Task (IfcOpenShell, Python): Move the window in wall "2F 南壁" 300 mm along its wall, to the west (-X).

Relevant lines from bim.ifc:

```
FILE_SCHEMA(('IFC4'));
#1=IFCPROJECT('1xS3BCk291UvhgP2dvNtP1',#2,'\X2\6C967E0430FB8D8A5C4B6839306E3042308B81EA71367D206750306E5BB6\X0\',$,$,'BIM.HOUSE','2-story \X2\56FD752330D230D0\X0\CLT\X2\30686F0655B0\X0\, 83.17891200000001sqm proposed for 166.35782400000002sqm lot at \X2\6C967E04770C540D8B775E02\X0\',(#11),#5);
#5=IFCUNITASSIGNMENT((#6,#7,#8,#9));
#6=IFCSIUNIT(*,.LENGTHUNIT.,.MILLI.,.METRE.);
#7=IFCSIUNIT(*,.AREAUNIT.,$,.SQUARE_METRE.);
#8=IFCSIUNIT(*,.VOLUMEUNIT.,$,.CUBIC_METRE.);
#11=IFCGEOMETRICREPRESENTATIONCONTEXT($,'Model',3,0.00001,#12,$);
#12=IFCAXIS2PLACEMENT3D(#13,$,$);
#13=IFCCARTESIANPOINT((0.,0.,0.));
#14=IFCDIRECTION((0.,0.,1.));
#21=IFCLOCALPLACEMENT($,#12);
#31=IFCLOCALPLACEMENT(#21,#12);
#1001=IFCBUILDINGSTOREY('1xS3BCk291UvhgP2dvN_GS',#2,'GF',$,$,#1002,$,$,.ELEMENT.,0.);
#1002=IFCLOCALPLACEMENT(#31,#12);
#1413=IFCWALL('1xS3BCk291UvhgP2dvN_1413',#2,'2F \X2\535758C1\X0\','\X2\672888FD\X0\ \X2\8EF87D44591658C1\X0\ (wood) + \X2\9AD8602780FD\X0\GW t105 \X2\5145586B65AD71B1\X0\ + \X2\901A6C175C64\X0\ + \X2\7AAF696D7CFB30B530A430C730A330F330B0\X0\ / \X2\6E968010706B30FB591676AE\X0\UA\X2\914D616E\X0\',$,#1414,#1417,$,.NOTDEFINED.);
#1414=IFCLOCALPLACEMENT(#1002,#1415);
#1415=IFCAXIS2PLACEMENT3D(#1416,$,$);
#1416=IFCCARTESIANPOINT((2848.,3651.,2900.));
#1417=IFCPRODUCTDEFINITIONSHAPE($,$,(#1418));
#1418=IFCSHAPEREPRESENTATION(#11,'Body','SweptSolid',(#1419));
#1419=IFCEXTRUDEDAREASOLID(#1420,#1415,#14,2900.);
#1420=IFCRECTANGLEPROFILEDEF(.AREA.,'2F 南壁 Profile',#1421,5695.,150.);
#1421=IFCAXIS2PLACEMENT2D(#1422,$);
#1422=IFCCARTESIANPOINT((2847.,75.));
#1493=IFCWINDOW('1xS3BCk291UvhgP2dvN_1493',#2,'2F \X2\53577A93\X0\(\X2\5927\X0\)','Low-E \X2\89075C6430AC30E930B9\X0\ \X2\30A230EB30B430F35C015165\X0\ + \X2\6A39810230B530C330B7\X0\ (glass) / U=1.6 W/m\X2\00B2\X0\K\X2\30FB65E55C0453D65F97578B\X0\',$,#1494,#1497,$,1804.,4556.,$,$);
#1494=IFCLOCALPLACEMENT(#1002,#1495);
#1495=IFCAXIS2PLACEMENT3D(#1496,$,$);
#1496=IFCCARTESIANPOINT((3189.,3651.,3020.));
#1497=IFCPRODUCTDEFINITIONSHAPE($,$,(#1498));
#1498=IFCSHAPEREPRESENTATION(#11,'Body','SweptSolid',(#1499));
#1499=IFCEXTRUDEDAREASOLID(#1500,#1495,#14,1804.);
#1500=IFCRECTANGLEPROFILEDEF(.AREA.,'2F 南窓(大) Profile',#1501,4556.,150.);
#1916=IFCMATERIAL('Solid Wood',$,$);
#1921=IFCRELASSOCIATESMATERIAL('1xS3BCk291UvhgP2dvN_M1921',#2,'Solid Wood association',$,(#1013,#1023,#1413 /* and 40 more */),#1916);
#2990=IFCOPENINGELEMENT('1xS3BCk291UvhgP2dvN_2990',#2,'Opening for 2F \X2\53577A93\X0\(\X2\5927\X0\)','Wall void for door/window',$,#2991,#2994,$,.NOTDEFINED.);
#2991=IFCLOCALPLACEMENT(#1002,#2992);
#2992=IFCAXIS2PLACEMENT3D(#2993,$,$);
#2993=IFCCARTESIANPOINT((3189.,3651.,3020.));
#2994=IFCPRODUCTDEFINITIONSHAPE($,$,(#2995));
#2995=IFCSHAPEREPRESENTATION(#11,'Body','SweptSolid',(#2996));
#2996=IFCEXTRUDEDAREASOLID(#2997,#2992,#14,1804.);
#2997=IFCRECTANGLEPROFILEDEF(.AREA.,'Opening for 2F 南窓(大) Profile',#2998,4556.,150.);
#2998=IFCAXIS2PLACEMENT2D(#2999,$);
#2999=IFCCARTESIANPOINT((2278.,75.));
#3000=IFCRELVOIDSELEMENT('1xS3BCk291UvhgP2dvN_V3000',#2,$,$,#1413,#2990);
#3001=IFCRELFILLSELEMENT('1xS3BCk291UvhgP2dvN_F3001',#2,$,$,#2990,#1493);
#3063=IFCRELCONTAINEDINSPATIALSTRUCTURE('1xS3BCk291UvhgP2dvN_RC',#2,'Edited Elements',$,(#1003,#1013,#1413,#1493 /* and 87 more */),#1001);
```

```python
import ifcopenshell
import ifcopenshell.api.geometry
import ifcopenshell.util.placement

model = ifcopenshell.open("bim.ifc")

window = model.by_id(1493)
opening = window.FillsVoids[0].RelatingOpeningElement
wall = opening.VoidsElements[0].RelatingBuildingElement

wall_matrix = ifcopenshell.util.placement.get_local_placement(wall.ObjectPlacement)
shift = wall_matrix[:3, 0] * -300.0
before = ifcopenshell.util.placement.get_local_placement(window.ObjectPlacement)[:3, 3].copy()

# The window is not placed relative to its opening, so move both.
for product in (opening, window):
    matrix = ifcopenshell.util.placement.get_local_placement(product.ObjectPlacement)
    matrix[:3, 3] += shift
    ifcopenshell.api.geometry.edit_object_placement(model, product=product, matrix=matrix, is_si=False)

after = ifcopenshell.util.placement.get_local_placement(window.ObjectPlacement)[:3, 3]
print("window moved by", (after - before).round(3) + 0.0)

model.write("bim_v2.ifc")
```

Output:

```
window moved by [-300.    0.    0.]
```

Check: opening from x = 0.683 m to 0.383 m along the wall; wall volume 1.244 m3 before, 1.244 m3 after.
